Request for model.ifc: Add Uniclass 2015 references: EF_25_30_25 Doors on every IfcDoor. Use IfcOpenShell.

First a look at what the model holds.

```python
import ifcopenshell

model = ifcopenshell.open("model.ifc")
print(model.schema)
print("classifications:", [c.Name for c in model.by_type("IfcClassification")])
for ifc_class in ("IfcDoor", "IfcRoof", "IfcStair", "IfcWall", "IfcWindow"):
    print(ifc_class, len(model.by_type(ifc_class)))
```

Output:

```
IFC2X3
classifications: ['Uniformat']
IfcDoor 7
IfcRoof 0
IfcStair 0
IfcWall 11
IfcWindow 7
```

```python
import ifcopenshell
import ifcopenshell.api.classification

model = ifcopenshell.open("model.ifc")

# IFC2X3 requires Source and Edition and has no link from the project to the system.
system = model.create_entity("IfcClassification", Source="NBS", Edition="2015", Name="Uniclass 2015")

codes = {
    "IfcDoor": ("EF_25_30_25", "Doors"),
}
for ifc_class, (code, name) in codes.items():
    products = model.by_type(ifc_class)
    ifcopenshell.api.classification.add_reference(
        model, products=products, classification=system, identification=code, name=name
    )
    print(code, len(products))

model.write("model_v2.ifc")
```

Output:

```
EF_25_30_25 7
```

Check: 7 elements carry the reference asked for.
